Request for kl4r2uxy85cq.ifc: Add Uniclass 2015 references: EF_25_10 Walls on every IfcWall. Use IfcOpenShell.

First a look at what the model holds.

```python
import ifcopenshell

model = ifcopenshell.open("kl4r2uxy85cq.ifc")
print(model.schema)
print("classifications:", [c.Name for c in model.by_type("IfcClassification")])
for ifc_class in ("IfcDoor", "IfcRoof", "IfcStair", "IfcWall", "IfcWindow"):
    print(ifc_class, len(model.by_type(ifc_class)))
```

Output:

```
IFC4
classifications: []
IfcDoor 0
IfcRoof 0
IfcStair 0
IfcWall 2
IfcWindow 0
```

```python
import ifcopenshell
import ifcopenshell.api.classification

model = ifcopenshell.open("kl4r2uxy85cq.ifc")

system = ifcopenshell.api.classification.add_classification(model, classification="Uniclass 2015")

codes = {
    "IfcWall": ("EF_25_10", "Walls"),
}
for ifc_class, (code, name) in codes.items():
    products = model.by_type(ifc_class)
    ifcopenshell.api.classification.add_reference(
        model, products=products, classification=system, identification=code, name=name
    )
    print(code, len(products))

model.write("kl4r2uxy85cq_rev.ifc")
```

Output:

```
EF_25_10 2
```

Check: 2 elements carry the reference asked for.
